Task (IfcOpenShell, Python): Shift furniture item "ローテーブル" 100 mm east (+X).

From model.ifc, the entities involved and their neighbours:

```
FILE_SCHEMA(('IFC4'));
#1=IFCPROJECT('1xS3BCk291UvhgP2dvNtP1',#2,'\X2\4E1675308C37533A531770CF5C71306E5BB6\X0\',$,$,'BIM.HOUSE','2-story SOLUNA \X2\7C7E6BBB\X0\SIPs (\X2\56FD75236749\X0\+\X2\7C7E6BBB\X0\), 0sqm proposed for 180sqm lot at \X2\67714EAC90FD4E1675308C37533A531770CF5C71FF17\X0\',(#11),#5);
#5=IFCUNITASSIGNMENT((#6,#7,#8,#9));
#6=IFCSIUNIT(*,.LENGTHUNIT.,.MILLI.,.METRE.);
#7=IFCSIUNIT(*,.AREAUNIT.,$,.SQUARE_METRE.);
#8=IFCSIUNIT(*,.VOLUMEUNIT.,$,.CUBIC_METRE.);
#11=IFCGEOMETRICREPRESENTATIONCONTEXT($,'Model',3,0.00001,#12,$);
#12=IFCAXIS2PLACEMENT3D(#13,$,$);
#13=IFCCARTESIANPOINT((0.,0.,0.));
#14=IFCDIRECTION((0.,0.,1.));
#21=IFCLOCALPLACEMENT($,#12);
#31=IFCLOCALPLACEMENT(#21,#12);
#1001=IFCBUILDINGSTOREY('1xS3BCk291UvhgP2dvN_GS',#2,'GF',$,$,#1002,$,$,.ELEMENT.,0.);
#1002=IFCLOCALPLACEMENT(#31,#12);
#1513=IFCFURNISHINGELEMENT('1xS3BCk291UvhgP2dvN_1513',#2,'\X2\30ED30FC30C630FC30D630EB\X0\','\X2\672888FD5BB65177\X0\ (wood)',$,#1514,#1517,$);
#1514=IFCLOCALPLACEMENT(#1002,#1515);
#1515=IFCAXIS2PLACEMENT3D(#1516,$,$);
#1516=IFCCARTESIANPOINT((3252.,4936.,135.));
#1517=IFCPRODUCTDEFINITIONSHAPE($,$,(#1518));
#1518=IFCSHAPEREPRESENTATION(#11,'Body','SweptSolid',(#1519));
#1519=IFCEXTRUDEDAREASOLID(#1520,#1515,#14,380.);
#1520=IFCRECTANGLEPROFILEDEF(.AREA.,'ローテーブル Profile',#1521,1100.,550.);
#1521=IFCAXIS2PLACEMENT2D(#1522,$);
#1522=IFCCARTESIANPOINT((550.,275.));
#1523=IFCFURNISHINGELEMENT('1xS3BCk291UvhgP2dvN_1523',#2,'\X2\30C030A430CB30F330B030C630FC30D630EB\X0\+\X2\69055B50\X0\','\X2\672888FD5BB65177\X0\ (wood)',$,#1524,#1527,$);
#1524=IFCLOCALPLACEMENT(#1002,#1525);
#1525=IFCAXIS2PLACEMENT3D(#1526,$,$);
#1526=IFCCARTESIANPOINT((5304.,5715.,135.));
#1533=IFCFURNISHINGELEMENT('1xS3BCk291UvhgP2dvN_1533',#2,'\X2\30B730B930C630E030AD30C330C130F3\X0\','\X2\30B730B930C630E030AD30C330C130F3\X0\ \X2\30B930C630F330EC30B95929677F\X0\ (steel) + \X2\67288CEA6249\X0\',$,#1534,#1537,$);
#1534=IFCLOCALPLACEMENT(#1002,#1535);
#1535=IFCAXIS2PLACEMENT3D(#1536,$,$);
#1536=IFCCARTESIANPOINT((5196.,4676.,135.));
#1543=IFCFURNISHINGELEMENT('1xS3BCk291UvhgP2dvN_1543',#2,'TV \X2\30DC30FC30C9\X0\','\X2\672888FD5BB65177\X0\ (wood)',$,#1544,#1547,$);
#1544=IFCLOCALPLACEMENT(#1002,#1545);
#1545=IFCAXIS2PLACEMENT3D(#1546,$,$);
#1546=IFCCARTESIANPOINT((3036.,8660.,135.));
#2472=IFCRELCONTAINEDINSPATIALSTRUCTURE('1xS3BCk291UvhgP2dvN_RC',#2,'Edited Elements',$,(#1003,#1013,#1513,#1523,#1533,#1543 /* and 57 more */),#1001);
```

```python
import ifcopenshell
import ifcopenshell.api.geometry
import ifcopenshell.util.placement
import ifcopenshell.util.unit

model = ifcopenshell.open("model.ifc")
unit_scale = ifcopenshell.util.unit.calculate_unit_scale(model)

item = model.by_guid("1xS3BCk291UvhgP2dvN_1513")
matrix = ifcopenshell.util.placement.get_local_placement(item.ObjectPlacement)
matrix[0, 3] += 0.1 / unit_scale
ifcopenshell.api.geometry.edit_object_placement(model, product=item, matrix=matrix, is_si=False)

print(ifcopenshell.util.placement.get_local_placement(item.ObjectPlacement).round(3) + 0.0)

model.write("model_edited.ifc")
```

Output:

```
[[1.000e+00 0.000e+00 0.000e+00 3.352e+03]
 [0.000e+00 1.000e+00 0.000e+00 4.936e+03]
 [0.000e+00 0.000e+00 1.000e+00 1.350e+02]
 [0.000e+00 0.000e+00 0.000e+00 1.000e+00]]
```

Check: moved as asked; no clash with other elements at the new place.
